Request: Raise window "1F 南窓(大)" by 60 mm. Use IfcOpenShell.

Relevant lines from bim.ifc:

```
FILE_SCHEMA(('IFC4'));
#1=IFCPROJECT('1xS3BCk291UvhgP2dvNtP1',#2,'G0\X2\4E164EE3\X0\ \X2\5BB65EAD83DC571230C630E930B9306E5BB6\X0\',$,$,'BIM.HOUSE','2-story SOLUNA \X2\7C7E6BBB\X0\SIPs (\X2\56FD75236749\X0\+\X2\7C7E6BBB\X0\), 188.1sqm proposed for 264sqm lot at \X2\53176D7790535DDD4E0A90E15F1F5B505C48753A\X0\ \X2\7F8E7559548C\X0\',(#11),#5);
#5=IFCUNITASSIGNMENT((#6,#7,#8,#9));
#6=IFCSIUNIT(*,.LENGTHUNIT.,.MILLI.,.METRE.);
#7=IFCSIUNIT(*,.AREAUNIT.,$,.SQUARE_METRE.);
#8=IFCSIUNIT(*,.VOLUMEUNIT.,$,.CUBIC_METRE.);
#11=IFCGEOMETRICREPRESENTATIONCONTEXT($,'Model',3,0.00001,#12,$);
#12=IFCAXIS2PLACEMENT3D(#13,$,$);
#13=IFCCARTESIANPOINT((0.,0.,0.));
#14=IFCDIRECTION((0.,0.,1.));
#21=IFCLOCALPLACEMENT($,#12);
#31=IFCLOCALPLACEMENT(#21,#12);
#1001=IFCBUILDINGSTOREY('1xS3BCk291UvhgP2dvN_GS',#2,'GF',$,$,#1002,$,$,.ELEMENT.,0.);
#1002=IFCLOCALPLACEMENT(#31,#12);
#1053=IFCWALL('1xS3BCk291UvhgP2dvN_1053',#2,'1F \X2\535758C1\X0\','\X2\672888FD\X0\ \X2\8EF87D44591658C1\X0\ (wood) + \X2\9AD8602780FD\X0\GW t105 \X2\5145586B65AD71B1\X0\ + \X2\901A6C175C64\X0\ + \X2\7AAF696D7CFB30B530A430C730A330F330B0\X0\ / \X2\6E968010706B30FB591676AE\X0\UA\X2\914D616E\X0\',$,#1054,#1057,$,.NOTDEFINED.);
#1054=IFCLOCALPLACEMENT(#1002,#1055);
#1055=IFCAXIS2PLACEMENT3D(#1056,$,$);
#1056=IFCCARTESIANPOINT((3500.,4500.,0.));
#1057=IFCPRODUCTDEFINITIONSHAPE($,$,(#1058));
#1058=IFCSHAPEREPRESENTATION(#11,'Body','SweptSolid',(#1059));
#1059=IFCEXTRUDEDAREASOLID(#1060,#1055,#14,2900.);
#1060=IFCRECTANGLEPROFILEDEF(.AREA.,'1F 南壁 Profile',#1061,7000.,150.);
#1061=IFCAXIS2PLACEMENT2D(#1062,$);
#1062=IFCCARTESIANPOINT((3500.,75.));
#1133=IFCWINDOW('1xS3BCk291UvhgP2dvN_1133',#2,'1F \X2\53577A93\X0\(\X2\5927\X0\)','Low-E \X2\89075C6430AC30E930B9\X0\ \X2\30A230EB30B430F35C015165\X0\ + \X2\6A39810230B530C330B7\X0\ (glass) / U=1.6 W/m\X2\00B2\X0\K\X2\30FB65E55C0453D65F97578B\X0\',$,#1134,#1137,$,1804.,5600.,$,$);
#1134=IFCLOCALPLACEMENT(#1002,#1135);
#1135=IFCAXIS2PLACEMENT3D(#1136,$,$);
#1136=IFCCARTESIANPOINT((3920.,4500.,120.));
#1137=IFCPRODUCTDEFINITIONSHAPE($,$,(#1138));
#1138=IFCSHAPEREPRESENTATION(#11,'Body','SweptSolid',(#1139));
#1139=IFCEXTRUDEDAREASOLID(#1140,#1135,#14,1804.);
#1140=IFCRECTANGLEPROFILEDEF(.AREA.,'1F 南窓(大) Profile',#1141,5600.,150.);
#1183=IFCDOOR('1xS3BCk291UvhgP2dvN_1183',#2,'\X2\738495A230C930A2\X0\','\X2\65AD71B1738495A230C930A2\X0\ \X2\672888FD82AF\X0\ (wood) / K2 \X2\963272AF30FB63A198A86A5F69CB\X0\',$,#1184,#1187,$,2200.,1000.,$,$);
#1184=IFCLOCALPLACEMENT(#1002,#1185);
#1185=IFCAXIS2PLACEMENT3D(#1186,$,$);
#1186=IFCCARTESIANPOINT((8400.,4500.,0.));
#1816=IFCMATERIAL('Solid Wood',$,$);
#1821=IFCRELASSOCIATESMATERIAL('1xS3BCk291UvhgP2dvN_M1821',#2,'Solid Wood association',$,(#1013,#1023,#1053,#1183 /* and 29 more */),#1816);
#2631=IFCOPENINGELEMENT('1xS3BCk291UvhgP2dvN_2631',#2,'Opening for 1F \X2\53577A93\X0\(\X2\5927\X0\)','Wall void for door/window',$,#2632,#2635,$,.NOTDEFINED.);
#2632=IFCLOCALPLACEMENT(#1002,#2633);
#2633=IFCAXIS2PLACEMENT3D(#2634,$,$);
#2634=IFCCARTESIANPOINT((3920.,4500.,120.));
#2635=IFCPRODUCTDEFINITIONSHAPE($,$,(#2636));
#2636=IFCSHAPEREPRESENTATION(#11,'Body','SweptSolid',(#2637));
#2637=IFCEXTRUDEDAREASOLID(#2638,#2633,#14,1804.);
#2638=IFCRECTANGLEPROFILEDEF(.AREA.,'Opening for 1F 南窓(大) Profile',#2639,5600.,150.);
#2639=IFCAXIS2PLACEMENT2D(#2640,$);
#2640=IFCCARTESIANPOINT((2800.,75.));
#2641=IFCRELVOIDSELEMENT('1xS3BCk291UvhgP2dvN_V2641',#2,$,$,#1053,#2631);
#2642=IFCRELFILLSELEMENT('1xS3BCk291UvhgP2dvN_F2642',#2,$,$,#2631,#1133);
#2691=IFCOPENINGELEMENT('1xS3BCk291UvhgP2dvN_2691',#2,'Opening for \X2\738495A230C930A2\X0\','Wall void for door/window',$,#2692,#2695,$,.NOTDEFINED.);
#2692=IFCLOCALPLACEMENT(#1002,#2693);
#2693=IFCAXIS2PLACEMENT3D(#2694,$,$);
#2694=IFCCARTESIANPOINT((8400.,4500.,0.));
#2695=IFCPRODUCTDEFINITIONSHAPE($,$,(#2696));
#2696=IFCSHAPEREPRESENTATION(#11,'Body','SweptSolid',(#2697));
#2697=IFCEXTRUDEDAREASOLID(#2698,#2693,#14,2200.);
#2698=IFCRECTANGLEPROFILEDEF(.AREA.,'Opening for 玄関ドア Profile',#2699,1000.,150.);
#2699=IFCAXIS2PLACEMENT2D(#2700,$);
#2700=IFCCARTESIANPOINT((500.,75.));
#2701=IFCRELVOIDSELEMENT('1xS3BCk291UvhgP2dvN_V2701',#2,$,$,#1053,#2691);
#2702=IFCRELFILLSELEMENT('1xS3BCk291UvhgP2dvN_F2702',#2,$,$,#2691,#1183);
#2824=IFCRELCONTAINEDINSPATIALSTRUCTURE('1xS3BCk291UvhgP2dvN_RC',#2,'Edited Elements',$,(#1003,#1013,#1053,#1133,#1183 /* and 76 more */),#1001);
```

```python
import numpy as np
import ifcopenshell
import ifcopenshell.api.geometry
import ifcopenshell.util.placement
import ifcopenshell.util.unit

model = ifcopenshell.open("bim.ifc")
unit_scale = ifcopenshell.util.unit.calculate_unit_scale(model)

window = model.by_guid("1xS3BCk291UvhgP2dvN_1133")
opening = window.FillsVoids[0].RelatingOpeningElement
dz = 60.0

shift = np.array([0.0, 0.0, dz])
# The window is not placed relative to its opening, so move both.
for product in (opening, window):
    matrix = ifcopenshell.util.placement.get_local_placement(product.ObjectPlacement)
    matrix[:3, 3] += shift
    ifcopenshell.api.geometry.edit_object_placement(model, product=product, matrix=matrix, is_si=False)

print(f"moved by {dz * unit_scale:+.3f} m")

model.write("bim_updated.ifc")
```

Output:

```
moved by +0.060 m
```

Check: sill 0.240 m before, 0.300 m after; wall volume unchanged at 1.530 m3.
